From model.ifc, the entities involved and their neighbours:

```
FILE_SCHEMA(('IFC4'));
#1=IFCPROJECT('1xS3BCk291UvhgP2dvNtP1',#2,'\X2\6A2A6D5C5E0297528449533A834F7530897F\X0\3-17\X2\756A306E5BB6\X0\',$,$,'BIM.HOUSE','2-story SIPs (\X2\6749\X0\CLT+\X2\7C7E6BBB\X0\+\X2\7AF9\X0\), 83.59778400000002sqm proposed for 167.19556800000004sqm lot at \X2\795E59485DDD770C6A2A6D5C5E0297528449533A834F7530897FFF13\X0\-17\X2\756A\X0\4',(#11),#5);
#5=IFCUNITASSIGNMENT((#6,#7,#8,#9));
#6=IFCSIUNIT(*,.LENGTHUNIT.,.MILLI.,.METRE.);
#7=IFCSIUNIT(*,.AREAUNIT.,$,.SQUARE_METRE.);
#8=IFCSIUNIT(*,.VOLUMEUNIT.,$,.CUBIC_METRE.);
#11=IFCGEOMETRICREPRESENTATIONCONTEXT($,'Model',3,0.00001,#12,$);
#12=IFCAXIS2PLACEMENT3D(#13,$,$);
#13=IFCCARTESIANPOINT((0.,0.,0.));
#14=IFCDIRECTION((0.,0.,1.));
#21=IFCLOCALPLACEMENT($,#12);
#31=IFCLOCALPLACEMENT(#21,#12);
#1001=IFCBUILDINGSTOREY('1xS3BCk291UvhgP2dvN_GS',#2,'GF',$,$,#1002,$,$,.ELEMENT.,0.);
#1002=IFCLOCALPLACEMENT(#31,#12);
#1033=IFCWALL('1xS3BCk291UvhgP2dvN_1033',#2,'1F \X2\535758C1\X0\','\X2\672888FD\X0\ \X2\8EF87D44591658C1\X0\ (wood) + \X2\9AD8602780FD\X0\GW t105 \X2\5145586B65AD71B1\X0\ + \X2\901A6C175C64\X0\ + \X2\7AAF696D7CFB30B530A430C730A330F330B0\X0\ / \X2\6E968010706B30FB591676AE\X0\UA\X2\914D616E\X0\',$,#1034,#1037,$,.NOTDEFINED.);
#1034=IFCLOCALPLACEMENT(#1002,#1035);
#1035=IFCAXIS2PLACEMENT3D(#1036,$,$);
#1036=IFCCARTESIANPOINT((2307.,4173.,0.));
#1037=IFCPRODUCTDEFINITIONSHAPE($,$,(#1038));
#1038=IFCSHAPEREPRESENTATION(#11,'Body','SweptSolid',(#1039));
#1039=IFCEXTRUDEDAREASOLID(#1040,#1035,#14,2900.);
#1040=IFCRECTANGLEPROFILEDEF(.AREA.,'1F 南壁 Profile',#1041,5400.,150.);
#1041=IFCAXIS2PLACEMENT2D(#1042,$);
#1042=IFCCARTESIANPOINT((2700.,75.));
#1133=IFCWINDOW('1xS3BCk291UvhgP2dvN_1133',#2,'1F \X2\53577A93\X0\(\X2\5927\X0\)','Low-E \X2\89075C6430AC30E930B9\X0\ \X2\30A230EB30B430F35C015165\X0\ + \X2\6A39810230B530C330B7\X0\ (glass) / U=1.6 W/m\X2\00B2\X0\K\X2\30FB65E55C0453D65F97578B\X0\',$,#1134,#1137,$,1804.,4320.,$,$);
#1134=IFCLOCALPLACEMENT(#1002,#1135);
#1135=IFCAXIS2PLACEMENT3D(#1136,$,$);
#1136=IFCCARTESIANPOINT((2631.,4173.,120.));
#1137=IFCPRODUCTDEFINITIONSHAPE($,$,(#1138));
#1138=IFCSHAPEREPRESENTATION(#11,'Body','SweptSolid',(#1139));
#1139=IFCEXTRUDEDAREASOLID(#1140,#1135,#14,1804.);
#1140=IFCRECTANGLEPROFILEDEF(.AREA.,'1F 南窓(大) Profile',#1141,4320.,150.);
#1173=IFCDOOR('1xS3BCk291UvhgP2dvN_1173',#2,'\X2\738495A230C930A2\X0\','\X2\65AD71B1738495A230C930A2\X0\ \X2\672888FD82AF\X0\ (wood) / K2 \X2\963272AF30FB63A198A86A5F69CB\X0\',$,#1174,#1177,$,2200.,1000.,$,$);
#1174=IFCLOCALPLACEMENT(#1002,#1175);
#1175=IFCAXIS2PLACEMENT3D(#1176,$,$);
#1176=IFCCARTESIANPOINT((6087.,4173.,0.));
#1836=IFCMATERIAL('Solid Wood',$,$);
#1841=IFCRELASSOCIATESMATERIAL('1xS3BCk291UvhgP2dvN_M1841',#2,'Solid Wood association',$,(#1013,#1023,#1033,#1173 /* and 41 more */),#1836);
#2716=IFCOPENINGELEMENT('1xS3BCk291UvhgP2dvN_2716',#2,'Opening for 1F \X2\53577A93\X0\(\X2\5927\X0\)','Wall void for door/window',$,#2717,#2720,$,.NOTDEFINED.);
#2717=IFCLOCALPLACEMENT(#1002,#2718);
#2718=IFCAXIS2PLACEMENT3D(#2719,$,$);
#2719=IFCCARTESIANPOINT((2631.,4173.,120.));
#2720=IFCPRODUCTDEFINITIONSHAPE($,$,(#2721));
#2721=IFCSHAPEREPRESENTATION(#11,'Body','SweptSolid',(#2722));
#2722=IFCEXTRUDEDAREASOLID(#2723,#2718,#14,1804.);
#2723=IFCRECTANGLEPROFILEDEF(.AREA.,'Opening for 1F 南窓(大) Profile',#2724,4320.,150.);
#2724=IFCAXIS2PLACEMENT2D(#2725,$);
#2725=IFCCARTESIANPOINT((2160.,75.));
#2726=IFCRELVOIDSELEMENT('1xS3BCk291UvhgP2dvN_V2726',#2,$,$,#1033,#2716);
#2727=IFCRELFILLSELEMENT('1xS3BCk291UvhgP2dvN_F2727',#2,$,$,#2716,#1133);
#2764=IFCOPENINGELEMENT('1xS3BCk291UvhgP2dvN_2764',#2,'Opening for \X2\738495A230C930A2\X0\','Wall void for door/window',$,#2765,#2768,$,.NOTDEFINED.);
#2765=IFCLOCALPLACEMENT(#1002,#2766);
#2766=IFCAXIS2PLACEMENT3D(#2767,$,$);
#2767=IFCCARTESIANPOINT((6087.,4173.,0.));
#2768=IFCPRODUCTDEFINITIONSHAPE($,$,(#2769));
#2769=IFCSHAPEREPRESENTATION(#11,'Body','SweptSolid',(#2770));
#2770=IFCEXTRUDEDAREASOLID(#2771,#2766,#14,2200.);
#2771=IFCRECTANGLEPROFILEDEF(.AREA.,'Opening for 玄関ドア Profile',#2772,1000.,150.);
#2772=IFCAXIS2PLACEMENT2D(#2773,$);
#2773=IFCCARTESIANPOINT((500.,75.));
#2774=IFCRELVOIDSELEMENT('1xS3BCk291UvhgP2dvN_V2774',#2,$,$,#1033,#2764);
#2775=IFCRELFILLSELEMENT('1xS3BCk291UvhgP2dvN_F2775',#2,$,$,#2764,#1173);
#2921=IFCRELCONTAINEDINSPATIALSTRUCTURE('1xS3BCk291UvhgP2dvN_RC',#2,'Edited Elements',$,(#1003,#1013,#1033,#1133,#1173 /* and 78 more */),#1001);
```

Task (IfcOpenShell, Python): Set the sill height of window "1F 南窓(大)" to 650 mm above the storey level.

```python
import numpy as np
import ifcopenshell
import ifcopenshell.api.geometry
import ifcopenshell.geom
import ifcopenshell.util.element
import ifcopenshell.util.placement
import ifcopenshell.util.shape
import ifcopenshell.util.unit

model = ifcopenshell.open("model.ifc")
unit_scale = ifcopenshell.util.unit.calculate_unit_scale(model)

window = model.by_id(1133)
opening = window.FillsVoids[0].RelatingOpeningElement
storey = ifcopenshell.util.element.get_container(window, ifc_class="IfcBuildingStorey")
level = ifcopenshell.util.placement.get_local_placement(storey.ObjectPlacement)[2, 3]

# The opening's origin need not be at the sill, so measure its lowest point.
shape = ifcopenshell.geom.create_shape(ifcopenshell.geom.settings(), opening)
bottom = ifcopenshell.util.shape.get_shape_bottom_elevation(shape, shape.geometry) / unit_scale
dz = level + 0.65 / unit_scale - bottom

shift = np.array([0.0, 0.0, dz])
# The window is not placed relative to its opening, so move both.
for product in (opening, window):
    matrix = ifcopenshell.util.placement.get_local_placement(product.ObjectPlacement)
    matrix[:3, 3] += shift
    ifcopenshell.api.geometry.edit_object_placement(model, product=product, matrix=matrix, is_si=False)

print(f"moved by {dz * unit_scale:+.3f} m")

model.write("model_v2.ifc")
```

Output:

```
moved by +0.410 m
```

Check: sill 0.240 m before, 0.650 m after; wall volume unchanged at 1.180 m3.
